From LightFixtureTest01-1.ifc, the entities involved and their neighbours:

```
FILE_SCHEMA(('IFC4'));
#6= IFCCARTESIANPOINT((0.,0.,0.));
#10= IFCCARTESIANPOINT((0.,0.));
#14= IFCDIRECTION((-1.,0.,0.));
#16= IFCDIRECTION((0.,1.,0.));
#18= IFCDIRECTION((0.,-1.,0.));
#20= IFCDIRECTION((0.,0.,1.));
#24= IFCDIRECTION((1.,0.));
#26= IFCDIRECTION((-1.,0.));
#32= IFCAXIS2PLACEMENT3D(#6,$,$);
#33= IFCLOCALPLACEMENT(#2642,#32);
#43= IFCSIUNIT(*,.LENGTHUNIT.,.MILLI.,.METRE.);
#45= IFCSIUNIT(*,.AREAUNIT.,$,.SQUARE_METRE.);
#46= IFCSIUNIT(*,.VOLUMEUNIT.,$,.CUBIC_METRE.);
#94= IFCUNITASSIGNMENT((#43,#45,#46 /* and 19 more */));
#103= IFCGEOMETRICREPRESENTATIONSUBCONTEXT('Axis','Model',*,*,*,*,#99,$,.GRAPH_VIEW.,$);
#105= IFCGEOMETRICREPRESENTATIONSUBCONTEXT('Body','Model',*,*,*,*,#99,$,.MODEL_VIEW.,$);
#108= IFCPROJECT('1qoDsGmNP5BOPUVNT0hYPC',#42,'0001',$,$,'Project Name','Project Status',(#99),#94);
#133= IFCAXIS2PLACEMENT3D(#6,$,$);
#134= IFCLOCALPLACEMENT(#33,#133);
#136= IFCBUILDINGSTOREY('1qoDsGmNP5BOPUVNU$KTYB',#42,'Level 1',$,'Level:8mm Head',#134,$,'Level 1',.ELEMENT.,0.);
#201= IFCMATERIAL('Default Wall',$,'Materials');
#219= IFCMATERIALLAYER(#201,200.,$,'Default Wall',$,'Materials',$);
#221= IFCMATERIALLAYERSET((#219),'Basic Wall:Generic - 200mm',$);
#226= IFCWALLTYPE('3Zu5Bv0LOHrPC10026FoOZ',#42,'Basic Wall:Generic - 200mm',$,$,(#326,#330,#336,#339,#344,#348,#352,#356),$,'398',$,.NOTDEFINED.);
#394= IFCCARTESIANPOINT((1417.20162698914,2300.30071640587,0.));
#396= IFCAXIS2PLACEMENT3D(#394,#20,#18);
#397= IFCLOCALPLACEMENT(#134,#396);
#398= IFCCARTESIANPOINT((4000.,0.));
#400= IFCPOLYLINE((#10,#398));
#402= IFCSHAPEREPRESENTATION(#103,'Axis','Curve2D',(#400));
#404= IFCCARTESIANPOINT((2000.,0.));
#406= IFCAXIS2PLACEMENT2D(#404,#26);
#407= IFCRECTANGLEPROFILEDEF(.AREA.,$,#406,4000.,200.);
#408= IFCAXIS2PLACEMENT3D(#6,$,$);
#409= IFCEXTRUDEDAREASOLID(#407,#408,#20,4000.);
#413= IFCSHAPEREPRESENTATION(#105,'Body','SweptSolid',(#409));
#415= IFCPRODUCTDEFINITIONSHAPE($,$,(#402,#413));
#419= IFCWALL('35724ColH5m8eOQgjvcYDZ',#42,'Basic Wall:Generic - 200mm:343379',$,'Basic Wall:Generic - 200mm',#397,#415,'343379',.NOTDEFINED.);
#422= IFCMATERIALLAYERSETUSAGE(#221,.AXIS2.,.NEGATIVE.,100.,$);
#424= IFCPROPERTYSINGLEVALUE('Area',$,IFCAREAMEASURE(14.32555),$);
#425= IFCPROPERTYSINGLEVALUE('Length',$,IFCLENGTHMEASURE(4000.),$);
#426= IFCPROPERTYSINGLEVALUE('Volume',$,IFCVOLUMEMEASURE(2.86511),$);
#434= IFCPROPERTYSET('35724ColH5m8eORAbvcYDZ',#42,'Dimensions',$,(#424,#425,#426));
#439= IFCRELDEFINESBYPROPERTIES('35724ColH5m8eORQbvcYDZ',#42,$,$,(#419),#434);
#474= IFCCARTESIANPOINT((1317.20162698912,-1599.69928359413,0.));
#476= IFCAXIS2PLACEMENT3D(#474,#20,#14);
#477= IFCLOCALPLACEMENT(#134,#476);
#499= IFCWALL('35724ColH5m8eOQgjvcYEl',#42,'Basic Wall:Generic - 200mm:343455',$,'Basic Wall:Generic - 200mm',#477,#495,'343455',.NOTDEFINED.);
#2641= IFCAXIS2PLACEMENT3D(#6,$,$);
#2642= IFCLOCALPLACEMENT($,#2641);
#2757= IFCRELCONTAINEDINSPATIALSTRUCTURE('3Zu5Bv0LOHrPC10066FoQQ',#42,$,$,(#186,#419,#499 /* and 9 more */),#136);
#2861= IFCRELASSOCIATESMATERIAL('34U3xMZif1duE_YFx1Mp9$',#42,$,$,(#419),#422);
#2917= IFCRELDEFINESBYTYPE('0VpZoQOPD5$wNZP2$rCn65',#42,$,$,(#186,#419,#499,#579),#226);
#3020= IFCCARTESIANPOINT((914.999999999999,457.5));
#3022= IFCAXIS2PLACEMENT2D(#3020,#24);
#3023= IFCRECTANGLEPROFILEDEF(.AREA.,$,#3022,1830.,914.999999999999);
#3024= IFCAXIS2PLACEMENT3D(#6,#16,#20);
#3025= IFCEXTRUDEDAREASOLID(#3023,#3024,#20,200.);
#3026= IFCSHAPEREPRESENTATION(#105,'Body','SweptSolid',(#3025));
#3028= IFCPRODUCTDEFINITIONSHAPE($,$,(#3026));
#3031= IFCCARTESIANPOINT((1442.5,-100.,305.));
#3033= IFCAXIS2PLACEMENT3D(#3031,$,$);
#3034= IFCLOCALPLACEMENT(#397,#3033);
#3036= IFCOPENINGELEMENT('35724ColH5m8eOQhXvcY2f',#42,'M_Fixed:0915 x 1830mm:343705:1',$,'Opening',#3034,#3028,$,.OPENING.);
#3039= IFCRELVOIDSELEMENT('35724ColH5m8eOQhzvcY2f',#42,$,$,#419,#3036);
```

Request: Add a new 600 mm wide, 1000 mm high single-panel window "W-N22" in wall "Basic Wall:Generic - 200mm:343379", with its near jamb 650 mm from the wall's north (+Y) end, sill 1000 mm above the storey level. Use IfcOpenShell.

```python
import numpy as np
import ifcopenshell
import ifcopenshell.api.feature
import ifcopenshell.api.geometry
import ifcopenshell.api.pset
import ifcopenshell.api.root
import ifcopenshell.api.spatial
import ifcopenshell.geom
import ifcopenshell.util.element
import ifcopenshell.util.placement
import ifcopenshell.util.representation
import ifcopenshell.util.shape
import ifcopenshell.util.unit

model = ifcopenshell.open("LightFixtureTest01-1.ifc")
unit_scale = ifcopenshell.util.unit.calculate_unit_scale(model)
area_scale = ifcopenshell.util.unit.calculate_unit_scale(model, "AREAUNIT")
volume_scale = ifcopenshell.util.unit.calculate_unit_scale(model, "VOLUMEUNIT")
settings = ifcopenshell.geom.settings()


def volume(element):
    """Net volume in cubic metres, openings subtracted."""
    shape = ifcopenshell.geom.create_shape(settings, element)
    return ifcopenshell.util.shape.get_volume(shape.geometry)


wall = model.by_guid("35724ColH5m8eOQgjvcYDZ")
storey = ifcopenshell.util.element.get_container(wall, ifc_class="IfcBuildingStorey")
context = ifcopenshell.util.representation.get_context(model, "Model", "Body", "MODEL_VIEW")
before = volume(wall)

width, height, from_end, sill = 0.6, 1, 0.65, 1  # metres

# The wall runs along its own X axis, and the end named is its -X end.
wall_shape = ifcopenshell.geom.create_shape(settings, wall)
x, y, z = ifcopenshell.util.shape.get_vertices(wall_shape.geometry).T
start = x.min() + from_end
face, thickness = float(y.min()), float(y.max() - y.min())
wall_matrix = ifcopenshell.util.placement.get_local_placement(wall.ObjectPlacement)
level = ifcopenshell.util.placement.get_local_placement(storey.ObjectPlacement)[2, 3]


def in_wall(x, y):
    """Placement at x, y metres in the wall's axes, at sill height."""
    matrix = wall_matrix.copy()
    matrix[:, 3] = wall_matrix @ np.array([x / unit_scale, y / unit_scale, 0.0, 1.0])
    matrix[2, 3] = level + sill / unit_scale
    return matrix


# Opening: a box that overshoots both wall faces by 50 mm.
opening = ifcopenshell.api.root.create_entity(model, ifc_class="IfcOpeningElement", predefined_type="OPENING")
box = ifcopenshell.api.geometry.add_wall_representation(
    model, context=context, length=width, height=height, thickness=thickness + 0.1
)
ifcopenshell.api.geometry.assign_representation(model, product=opening, representation=box)
ifcopenshell.api.geometry.edit_object_placement(model, product=opening, matrix=in_wall(start, face - 0.05), is_si=False)
ifcopenshell.api.feature.add_feature(model, feature=opening, element=wall)

window = ifcopenshell.api.root.create_entity(model, ifc_class="IfcWindow", name="W-N22", predefined_type="WINDOW")
window.OverallWidth, window.OverallHeight = width / unit_scale, height / unit_scale
window.PartitioningType = "SINGLE_PANEL"
body = ifcopenshell.api.geometry.add_window_representation(
    model,
    context=context,
    overall_width=window.OverallWidth,
    overall_height=window.OverallHeight,
    partition_type="SINGLE_PANEL",
)
ifcopenshell.api.geometry.assign_representation(model, product=window, representation=body)
ifcopenshell.api.spatial.assign_container(model, products=[window], relating_structure=storey)
ifcopenshell.api.feature.add_filling(model, opening=opening, element=window)

# Centre the window in the wall's thickness.
ifcopenshell.api.geometry.edit_object_placement(model, product=window, matrix=in_wall(start, face), is_si=False)
window_shape = ifcopenshell.geom.create_shape(settings, window)
depth = ifcopenshell.util.shape.get_vertices(window_shape.geometry)[:, 1]
offset = face + thickness / 2 - (depth.min() + depth.max()) / 2
ifcopenshell.api.geometry.edit_object_placement(model, product=window, matrix=in_wall(start, offset), is_si=False)

after = volume(wall)

# Update the wall's stored quantities.
pset = model.by_id(ifcopenshell.util.element.get_pset(wall, "Dimensions", should_inherit=False)["id"])
ifcopenshell.api.pset.edit_pset(model, pset=pset, properties={
    "Area": model.create_entity("IfcAreaMeasure", after / thickness / area_scale),
    "Volume": model.create_entity("IfcVolumeMeasure", after / volume_scale),
})

print(f"wall volume {before:.3f} -> {after:.3f} m3")

model.write("LightFixtureTest01-1_v2.ifc")
```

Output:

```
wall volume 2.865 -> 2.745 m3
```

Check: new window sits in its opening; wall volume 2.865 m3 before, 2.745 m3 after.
